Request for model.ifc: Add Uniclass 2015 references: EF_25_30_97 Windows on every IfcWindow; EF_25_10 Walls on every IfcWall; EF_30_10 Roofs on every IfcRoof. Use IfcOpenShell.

First a look at what the model holds.

```python
import ifcopenshell

model = ifcopenshell.open("model.ifc")
print(model.schema)
print("classifications:", [c.Name for c in model.by_type("IfcClassification")])
for ifc_class in ("IfcDoor", "IfcRoof", "IfcStair", "IfcWall", "IfcWindow"):
    print(ifc_class, len(model.by_type(ifc_class)))
```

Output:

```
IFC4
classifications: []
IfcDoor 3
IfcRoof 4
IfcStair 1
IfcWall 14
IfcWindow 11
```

```python
import ifcopenshell
import ifcopenshell.api.classification

model = ifcopenshell.open("model.ifc")

system = ifcopenshell.api.classification.add_classification(model, classification="Uniclass 2015")

codes = {
    "IfcWindow": ("EF_25_30_97", "Windows"),
    "IfcWall": ("EF_25_10", "Walls"),
    "IfcRoof": ("EF_30_10", "Roofs"),
}
for ifc_class, (code, name) in codes.items():
    products = model.by_type(ifc_class)
    ifcopenshell.api.classification.add_reference(
        model, products=products, classification=system, identification=code, name=name
    )
    print(code, len(products))

model.write("model_edited.ifc")
```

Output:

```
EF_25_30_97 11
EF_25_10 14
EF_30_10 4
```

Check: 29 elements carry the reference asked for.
